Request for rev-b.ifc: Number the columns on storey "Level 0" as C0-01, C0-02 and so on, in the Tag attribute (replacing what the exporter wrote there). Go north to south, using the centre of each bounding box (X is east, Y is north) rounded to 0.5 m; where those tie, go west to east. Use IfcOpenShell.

First a look at what the model holds.

```python
import ifcopenshell
import ifcopenshell.util.element
import ifcopenshell.util.placement

model = ifcopenshell.open("rev-b.ifc")
print(model.schema)
storey = next(s for s in model.by_type("IfcBuildingStorey") if s.Name == "Level 0")
columns = [e for e in ifcopenshell.util.element.get_decomposition(storey) if e.is_a("IfcColumn")]
for e in sorted(columns, key=lambda e: e.id()):
    origin = ifcopenshell.util.placement.get_local_placement(e.ObjectPlacement)[:3, 3]
    print(e.id(), e.Tag, e.Name, origin.round(2) + 0.0, sep=" | ")
```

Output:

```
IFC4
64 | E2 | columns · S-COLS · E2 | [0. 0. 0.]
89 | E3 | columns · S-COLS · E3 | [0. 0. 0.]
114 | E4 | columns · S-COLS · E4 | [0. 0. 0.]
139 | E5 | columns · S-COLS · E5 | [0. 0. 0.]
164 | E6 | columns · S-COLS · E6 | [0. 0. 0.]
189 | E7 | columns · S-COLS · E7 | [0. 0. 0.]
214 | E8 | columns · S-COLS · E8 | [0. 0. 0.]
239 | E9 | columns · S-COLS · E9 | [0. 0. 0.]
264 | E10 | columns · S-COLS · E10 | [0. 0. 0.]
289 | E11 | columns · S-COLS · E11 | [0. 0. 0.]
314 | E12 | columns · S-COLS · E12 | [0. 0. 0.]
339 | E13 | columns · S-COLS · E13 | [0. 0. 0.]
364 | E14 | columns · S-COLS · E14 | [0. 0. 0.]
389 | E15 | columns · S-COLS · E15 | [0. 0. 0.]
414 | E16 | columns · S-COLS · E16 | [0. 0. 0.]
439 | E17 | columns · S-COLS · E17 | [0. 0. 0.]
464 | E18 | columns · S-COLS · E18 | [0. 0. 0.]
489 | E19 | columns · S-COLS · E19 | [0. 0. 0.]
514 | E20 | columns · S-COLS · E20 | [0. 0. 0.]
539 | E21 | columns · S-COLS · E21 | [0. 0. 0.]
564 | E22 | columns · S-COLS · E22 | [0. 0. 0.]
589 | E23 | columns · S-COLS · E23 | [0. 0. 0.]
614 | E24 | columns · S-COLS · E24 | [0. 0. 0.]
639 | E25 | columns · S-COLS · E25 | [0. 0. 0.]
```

```python
import ifcopenshell
import ifcopenshell.geom
import ifcopenshell.util.element
import ifcopenshell.util.shape

model = ifcopenshell.open("rev-b.ifc")
settings = ifcopenshell.geom.settings()
settings.set("use-world-coords", True)


def centre(element):
    shape = ifcopenshell.geom.create_shape(settings, element)
    return ifcopenshell.util.shape.get_bbox_centroid(shape.geometry)


storey = next(s for s in model.by_type("IfcBuildingStorey") if s.Name == "Level 0")
columns = [e for e in ifcopenshell.util.element.get_decomposition(storey) if e.is_a("IfcColumn")]

# Insertion points can sit at a corner or the storey origin, so sort by the geometry (in metres).
centres = {e: centre(e) for e in columns}
columns.sort(key=lambda e: (-round(centres[e][1] / 0.5), centres[e][0]))

for i, e in enumerate(columns, start=1):
    number = f"C0-{i:02d}"
    e.Tag = number
    print(e.id(), number)

model.write("rev-b_edited.ifc")
```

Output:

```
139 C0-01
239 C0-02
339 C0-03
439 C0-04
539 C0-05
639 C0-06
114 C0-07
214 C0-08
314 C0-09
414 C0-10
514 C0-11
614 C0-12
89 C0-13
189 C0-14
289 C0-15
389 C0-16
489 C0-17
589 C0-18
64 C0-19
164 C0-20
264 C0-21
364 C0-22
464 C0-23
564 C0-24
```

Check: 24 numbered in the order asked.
